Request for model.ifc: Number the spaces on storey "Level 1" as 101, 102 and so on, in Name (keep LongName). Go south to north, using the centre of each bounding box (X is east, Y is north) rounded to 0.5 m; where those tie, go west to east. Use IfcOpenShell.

First a look at what the model holds.

```python
import ifcopenshell
import ifcopenshell.util.element
import ifcopenshell.util.placement

model = ifcopenshell.open("model.ifc")
print(model.schema)
storey = next(s for s in model.by_type("IfcBuildingStorey") if s.Name == "Level 1")
spaces = [e for e in ifcopenshell.util.element.get_decomposition(storey) if e.is_a("IfcSpace")]
for e in sorted(spaces, key=lambda e: e.id()):
    origin = ifcopenshell.util.placement.get_local_placement(e.ObjectPlacement)[:3, 3]
    print(e.id(), e.Name, e.LongName, origin.round(2) + 0.0, sep=" | ")
```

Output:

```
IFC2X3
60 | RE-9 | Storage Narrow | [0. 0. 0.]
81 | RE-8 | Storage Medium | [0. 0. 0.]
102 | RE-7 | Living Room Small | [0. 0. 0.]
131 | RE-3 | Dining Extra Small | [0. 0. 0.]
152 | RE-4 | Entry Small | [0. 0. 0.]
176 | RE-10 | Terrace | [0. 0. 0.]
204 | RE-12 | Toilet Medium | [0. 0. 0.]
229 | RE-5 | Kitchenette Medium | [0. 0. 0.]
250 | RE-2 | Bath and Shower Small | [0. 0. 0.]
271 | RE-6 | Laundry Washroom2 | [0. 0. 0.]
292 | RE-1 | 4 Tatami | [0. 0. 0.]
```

```python
import ifcopenshell
import ifcopenshell.geom
import ifcopenshell.util.element
import ifcopenshell.util.shape

model = ifcopenshell.open("model.ifc")
settings = ifcopenshell.geom.settings()
settings.set("use-world-coords", True)


def centre(element):
    shape = ifcopenshell.geom.create_shape(settings, element)
    return ifcopenshell.util.shape.get_bbox_centroid(shape.geometry)


storey = next(s for s in model.by_type("IfcBuildingStorey") if s.Name == "Level 1")
spaces = [e for e in ifcopenshell.util.element.get_decomposition(storey) if e.is_a("IfcSpace")]

# Insertion points can sit at a corner or the storey origin, so sort by the geometry (in metres).
centres = {e: centre(e) for e in spaces}
spaces.sort(key=lambda e: (round(centres[e][1] / 0.5), centres[e][0]))

for i, e in enumerate(spaces, start=1):
    number = f"1{i:02d}"
    e.Name = number
    print(e.id(), number)

model.write("model-out.ifc")
```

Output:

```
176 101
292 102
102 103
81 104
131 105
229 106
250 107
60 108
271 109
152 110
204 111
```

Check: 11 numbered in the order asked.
